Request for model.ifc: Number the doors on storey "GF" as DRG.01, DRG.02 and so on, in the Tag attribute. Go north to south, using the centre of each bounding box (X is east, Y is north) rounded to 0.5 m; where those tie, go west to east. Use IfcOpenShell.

First a look at what the model holds.

```python
import ifcopenshell
import ifcopenshell.util.element
import ifcopenshell.util.placement

model = ifcopenshell.open("model.ifc")
print(model.schema)
storey = next(s for s in model.by_type("IfcBuildingStorey") if s.Name == "GF")
doors = [e for e in ifcopenshell.util.element.get_decomposition(storey) if e.is_a("IfcDoor")]
for e in sorted(doors, key=lambda e: e.id()):
    origin = ifcopenshell.util.placement.get_local_placement(e.ObjectPlacement)[:3, 3]
    print(e.id(), e.Tag, e.Name, origin.round(2) + 0.0, sep=" | ")
```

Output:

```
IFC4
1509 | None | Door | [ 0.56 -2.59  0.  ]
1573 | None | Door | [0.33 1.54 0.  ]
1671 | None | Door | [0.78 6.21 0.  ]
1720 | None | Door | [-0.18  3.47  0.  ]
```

```python
import ifcopenshell
import ifcopenshell.geom
import ifcopenshell.util.element
import ifcopenshell.util.shape

model = ifcopenshell.open("model.ifc")
settings = ifcopenshell.geom.settings()
settings.set("use-world-coords", True)


def centre(element):
    shape = ifcopenshell.geom.create_shape(settings, element)
    return ifcopenshell.util.shape.get_bbox_centroid(shape.geometry)


storey = next(s for s in model.by_type("IfcBuildingStorey") if s.Name == "GF")
doors = [e for e in ifcopenshell.util.element.get_decomposition(storey) if e.is_a("IfcDoor")]

# Insertion points can sit at a corner or the storey origin, so sort by the geometry (in metres).
centres = {e: centre(e) for e in doors}
doors.sort(key=lambda e: (-round(centres[e][1] / 0.5), centres[e][0]))

for i, e in enumerate(doors, start=1):
    number = f"DRG.{i:02d}"
    e.Tag = number
    print(e.id(), number)

model.write("model_edited.ifc")
```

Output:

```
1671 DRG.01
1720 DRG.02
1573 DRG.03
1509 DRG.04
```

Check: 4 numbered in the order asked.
